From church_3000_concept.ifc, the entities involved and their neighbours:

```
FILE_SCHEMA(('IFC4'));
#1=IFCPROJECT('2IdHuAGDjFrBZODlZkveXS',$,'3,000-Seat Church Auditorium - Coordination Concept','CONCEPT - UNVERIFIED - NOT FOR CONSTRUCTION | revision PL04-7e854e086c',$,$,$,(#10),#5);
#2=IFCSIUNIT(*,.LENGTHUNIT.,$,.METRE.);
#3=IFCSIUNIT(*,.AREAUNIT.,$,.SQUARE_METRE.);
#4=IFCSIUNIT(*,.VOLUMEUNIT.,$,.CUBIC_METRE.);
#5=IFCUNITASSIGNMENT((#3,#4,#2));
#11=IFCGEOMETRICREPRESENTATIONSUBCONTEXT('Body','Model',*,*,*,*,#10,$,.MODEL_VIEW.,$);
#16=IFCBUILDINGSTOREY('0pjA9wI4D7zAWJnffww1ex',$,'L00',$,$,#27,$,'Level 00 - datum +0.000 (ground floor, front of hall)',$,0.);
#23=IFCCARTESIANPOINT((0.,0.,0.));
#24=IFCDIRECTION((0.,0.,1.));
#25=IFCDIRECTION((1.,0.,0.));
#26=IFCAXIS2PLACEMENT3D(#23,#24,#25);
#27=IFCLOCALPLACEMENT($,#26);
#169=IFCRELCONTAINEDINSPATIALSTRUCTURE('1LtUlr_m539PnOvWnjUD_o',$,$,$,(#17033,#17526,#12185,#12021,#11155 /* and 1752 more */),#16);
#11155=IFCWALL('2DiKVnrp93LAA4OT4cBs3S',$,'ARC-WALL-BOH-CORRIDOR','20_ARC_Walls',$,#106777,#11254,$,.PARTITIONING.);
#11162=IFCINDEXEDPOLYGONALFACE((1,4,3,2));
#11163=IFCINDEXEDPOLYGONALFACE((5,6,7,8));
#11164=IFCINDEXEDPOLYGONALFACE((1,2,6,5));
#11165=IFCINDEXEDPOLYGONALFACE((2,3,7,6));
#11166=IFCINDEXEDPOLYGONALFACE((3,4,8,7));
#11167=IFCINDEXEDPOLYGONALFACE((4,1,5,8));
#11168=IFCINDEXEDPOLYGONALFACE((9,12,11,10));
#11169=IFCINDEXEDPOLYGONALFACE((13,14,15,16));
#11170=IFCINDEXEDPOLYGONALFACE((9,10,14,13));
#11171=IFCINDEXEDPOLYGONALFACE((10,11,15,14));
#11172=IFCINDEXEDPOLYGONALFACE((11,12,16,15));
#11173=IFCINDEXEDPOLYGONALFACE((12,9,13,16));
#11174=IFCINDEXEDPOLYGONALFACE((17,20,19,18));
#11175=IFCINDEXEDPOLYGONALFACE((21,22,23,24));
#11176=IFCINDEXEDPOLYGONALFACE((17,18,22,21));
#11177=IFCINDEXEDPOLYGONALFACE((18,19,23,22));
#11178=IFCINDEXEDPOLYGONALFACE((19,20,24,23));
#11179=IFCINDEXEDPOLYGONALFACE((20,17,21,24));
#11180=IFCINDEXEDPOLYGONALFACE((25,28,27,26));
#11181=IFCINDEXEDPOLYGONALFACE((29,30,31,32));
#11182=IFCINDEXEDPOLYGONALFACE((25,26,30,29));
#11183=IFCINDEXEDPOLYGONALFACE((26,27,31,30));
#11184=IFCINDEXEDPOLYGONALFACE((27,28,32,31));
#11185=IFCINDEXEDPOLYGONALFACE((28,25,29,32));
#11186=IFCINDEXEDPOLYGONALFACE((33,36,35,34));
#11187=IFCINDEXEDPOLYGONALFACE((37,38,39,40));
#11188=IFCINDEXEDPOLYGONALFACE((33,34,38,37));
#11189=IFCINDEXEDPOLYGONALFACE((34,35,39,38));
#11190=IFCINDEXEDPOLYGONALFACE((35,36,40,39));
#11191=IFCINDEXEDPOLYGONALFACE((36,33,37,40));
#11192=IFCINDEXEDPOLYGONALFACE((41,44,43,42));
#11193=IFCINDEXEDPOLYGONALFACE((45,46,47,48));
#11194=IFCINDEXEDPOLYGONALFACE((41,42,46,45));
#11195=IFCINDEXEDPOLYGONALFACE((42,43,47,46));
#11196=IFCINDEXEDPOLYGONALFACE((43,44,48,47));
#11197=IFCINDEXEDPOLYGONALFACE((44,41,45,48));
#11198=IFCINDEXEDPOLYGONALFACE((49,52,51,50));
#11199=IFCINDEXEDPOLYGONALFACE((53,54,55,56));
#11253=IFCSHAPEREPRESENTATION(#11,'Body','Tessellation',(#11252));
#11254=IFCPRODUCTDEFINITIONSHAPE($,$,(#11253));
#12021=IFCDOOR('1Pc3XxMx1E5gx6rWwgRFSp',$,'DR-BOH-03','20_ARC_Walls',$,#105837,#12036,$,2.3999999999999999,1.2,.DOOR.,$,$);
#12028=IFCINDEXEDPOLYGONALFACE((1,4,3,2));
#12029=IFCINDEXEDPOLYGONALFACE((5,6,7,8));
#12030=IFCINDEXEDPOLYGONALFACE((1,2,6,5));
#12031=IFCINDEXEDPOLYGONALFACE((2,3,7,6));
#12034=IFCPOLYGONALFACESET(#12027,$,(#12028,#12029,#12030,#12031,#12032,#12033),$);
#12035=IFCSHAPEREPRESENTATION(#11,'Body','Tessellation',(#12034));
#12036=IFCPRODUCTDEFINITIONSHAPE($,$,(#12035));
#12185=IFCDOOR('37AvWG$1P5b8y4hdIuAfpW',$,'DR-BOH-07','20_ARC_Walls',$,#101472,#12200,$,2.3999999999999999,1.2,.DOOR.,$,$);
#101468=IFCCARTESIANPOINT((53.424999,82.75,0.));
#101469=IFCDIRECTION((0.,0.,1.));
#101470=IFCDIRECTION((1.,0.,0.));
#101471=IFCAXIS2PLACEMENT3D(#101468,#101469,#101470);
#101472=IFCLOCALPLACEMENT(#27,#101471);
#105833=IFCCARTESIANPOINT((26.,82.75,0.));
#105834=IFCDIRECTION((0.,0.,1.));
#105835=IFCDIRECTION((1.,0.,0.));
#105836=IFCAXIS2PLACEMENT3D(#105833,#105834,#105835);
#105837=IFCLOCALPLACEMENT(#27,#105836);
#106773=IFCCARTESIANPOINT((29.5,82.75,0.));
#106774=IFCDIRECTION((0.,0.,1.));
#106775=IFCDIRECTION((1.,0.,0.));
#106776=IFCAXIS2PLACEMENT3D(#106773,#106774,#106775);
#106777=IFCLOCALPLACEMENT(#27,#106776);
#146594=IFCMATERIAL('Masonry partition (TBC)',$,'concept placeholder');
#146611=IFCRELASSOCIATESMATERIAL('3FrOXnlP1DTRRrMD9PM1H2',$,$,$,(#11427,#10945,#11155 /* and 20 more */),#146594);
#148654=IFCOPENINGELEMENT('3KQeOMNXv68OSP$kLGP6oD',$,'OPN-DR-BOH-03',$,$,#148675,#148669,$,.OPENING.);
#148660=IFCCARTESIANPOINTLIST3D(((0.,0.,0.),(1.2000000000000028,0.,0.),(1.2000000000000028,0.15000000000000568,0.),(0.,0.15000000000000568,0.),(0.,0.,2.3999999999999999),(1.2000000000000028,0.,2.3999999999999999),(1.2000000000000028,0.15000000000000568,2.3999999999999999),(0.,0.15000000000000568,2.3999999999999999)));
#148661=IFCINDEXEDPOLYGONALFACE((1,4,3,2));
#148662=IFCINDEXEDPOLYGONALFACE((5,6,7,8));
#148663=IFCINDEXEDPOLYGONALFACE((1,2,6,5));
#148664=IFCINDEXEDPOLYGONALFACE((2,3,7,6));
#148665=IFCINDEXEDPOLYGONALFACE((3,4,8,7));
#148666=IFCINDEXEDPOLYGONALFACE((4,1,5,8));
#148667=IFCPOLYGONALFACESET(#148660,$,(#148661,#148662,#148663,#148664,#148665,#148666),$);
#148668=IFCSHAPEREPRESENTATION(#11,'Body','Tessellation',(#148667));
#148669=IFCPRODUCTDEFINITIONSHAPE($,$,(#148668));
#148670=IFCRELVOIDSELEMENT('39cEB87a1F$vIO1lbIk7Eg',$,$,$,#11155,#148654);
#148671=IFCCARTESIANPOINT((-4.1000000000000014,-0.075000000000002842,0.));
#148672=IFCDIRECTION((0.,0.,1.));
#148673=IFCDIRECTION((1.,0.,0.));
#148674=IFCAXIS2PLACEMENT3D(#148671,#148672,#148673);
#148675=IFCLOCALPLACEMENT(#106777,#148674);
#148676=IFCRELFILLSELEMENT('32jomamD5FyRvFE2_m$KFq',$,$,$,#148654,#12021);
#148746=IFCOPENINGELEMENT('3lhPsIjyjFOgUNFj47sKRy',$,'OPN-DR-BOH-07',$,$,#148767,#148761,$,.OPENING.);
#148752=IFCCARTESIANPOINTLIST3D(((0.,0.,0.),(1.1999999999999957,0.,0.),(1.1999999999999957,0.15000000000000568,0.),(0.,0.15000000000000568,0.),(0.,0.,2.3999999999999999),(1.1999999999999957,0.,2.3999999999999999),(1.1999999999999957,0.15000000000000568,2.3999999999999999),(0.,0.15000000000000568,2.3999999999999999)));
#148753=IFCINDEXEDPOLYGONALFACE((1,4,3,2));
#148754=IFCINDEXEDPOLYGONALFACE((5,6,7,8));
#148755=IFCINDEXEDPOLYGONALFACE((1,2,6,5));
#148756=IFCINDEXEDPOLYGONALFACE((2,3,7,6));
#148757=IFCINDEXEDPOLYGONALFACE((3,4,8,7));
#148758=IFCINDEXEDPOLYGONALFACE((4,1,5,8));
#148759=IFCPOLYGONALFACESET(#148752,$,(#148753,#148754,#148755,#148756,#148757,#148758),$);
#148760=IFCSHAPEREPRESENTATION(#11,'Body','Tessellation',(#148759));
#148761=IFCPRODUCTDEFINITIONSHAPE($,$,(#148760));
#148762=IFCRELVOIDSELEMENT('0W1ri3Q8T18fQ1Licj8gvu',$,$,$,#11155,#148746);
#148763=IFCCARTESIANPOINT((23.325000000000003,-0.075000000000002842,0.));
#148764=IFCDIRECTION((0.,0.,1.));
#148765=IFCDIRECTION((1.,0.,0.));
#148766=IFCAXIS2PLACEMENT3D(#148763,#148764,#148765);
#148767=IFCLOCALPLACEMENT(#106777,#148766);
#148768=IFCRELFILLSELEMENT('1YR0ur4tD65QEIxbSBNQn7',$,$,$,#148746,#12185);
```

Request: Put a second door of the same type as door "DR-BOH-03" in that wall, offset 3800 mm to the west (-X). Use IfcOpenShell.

```python
import ifcopenshell
import ifcopenshell.api.feature
import ifcopenshell.api.geometry
import ifcopenshell.api.root
import ifcopenshell.geom
import ifcopenshell.util.element
import ifcopenshell.util.placement
import ifcopenshell.util.shape

model = ifcopenshell.open("church_3000_concept.ifc")
settings = ifcopenshell.geom.settings()


def volume(element):
    """Net volume in cubic metres, openings subtracted."""
    shape = ifcopenshell.geom.create_shape(settings, element)
    return ifcopenshell.util.shape.get_volume(shape.geometry)


door = model.by_guid("1Pc3XxMx1E5gx6rWwgRFSp")
opening = door.FillsVoids[0].RelatingOpeningElement
wall = opening.VoidsElements[0].RelatingBuildingElement
before = volume(wall)
shift = ifcopenshell.util.placement.get_local_placement(wall.ObjectPlacement)[:3, 0] * -3.8

# copy_class copies the void relationship, type, container and properties, but no geometry.
new_opening = ifcopenshell.api.root.copy_class(model, product=opening)
new_opening.Representation = ifcopenshell.util.element.copy_deep(
    model, opening.Representation, exclude=["IfcGeometricRepresentationContext", "IfcRepresentationMap"]
)
new_door = ifcopenshell.api.root.copy_class(model, product=door)
new_door.Representation = ifcopenshell.util.element.copy_deep(
    model, door.Representation, exclude=["IfcGeometricRepresentationContext", "IfcRepresentationMap"]
)
ifcopenshell.api.feature.add_filling(model, opening=new_opening, element=new_door)

for old, new in ((opening, new_opening), (door, new_door)):
    matrix = ifcopenshell.util.placement.get_local_placement(old.ObjectPlacement)
    matrix[:3, 3] += shift
    ifcopenshell.api.geometry.edit_object_placement(model, product=new, matrix=matrix, is_si=False)

after = volume(wall)

print(f"wall volume {before:.3f} -> {after:.3f} m3")

model.write("church_3000_concept_v2.ifc")
```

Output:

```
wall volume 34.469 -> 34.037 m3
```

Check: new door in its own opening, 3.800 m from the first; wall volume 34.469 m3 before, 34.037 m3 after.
